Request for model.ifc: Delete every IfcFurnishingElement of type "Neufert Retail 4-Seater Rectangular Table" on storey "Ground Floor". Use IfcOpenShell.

First a look at what the model holds.

```python
import ifcopenshell
import ifcopenshell.util.element

model = ifcopenshell.open("model.ifc")
print(model.schema)
storey = next(s for s in model.by_type("IfcBuildingStorey") if s.Name == "Ground Floor")
furniture = [e for e in ifcopenshell.util.element.get_decomposition(storey) if e.is_a("IfcFurnishingElement")]
seen = {}
for e in furniture:
    element_type = ifcopenshell.util.element.get_type(e)
    name = element_type.Name if element_type not in (None, e) else None
    seen[name] = seen.get(name, 0) + 1
for name, count in sorted(seen.items(), key=str):
    print(count, "x", name)
```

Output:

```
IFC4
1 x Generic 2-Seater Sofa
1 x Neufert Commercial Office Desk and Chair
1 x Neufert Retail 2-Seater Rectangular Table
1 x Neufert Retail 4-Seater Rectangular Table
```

```python
import ifcopenshell
import ifcopenshell.api.root
import ifcopenshell.util.element

model = ifcopenshell.open("model.ifc")

storey = next(s for s in model.by_type("IfcBuildingStorey") if s.Name == "Ground Floor")
furniture = [e for e in ifcopenshell.util.element.get_decomposition(storey) if e.is_a("IfcFurnishingElement")]
targets = [e for e in furniture if (t := ifcopenshell.util.element.get_type(e)) not in (None, e) and t.Name == "Neufert Retail 4-Seater Rectangular Table"]

for e in targets:
    ifcopenshell.api.root.remove_product(model, product=e)
print(len(targets), "removed")

model.write("model_rev.ifc")
```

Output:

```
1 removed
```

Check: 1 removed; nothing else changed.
